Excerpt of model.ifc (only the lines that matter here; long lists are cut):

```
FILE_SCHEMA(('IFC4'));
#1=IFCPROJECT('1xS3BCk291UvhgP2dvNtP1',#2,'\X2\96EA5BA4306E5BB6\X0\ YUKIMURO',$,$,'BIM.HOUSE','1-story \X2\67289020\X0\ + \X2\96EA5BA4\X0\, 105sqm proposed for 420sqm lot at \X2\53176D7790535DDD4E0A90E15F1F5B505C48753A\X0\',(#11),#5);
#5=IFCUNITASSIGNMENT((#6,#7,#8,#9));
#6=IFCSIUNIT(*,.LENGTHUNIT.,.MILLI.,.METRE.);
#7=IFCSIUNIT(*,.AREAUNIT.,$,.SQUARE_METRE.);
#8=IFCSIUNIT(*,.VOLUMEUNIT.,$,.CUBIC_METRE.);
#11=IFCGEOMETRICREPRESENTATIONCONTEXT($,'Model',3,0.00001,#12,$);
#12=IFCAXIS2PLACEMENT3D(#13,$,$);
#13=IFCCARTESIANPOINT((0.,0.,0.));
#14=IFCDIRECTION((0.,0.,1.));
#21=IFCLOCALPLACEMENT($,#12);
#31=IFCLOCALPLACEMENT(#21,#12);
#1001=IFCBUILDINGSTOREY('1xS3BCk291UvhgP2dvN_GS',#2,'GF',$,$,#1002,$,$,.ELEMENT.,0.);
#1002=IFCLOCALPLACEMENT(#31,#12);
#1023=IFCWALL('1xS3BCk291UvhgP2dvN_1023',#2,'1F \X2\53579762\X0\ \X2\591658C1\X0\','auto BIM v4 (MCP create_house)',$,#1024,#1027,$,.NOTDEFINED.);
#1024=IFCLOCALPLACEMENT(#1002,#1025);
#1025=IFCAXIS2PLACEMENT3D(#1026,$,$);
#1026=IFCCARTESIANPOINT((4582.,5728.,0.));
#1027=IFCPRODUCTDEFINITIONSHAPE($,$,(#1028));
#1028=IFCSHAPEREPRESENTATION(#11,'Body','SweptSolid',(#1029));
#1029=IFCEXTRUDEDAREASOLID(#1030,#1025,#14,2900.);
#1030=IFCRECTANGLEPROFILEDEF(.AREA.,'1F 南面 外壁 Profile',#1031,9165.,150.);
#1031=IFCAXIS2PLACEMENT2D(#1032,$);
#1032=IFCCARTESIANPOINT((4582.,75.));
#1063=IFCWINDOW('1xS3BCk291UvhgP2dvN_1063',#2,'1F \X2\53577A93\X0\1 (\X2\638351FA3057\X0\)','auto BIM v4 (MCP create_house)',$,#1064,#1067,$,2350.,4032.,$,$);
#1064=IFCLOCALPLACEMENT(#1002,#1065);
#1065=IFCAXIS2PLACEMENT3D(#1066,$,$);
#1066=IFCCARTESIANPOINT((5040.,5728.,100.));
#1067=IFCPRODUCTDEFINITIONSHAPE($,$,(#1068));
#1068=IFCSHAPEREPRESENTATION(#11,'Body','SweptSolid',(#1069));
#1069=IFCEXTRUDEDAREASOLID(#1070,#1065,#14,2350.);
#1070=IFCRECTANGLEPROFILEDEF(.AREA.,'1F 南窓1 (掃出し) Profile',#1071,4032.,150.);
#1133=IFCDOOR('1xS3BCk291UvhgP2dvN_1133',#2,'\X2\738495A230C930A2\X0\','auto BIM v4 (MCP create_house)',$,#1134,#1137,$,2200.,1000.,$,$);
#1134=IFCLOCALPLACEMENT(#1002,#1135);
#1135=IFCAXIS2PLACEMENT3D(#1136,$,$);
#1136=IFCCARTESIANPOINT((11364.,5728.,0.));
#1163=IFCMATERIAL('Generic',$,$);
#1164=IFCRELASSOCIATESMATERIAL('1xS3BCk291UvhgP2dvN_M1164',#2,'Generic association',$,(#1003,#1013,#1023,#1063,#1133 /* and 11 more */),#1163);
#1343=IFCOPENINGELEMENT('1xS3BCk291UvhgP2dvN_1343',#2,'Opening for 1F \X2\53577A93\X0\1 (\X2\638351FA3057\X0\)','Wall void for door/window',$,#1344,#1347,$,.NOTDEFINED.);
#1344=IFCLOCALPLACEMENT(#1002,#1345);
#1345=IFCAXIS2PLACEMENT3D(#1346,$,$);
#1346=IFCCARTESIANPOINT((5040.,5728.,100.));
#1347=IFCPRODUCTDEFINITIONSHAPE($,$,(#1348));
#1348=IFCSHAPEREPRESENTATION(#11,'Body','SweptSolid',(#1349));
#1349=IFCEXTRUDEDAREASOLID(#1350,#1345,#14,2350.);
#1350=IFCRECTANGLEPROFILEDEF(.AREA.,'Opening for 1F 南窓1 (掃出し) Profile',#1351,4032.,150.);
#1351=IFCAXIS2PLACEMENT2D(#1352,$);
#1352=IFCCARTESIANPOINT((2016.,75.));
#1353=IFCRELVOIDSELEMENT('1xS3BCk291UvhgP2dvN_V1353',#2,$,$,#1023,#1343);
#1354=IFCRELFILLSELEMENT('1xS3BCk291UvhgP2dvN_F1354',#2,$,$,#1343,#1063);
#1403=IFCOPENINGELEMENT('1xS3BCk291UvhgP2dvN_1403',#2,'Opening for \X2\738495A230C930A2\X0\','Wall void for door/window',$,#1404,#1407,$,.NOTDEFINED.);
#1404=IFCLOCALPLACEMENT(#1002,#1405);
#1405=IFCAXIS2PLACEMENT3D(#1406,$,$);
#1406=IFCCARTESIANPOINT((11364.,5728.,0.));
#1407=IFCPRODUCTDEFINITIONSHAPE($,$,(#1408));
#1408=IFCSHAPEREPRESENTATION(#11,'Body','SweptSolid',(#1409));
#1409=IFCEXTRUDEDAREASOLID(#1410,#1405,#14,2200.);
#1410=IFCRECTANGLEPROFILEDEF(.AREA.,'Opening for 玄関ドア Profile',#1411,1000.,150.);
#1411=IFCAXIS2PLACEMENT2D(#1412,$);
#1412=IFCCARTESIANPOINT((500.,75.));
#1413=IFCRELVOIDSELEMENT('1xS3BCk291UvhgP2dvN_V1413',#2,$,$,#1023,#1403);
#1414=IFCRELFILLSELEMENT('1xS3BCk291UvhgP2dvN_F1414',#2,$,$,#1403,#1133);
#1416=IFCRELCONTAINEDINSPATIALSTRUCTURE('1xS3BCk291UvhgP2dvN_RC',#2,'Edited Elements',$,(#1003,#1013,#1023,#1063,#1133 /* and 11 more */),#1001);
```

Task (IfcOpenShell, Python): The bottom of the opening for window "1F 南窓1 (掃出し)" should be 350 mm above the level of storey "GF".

```python
import numpy as np
import ifcopenshell
import ifcopenshell.api.geometry
import ifcopenshell.geom
import ifcopenshell.util.element
import ifcopenshell.util.placement
import ifcopenshell.util.shape
import ifcopenshell.util.unit

model = ifcopenshell.open("model.ifc")
unit_scale = ifcopenshell.util.unit.calculate_unit_scale(model)

window = model.by_guid("1xS3BCk291UvhgP2dvN_1063")
opening = window.FillsVoids[0].RelatingOpeningElement
storey = ifcopenshell.util.element.get_container(window, ifc_class="IfcBuildingStorey")
level = ifcopenshell.util.placement.get_local_placement(storey.ObjectPlacement)[2, 3]

# The opening's origin need not be at the sill, so measure its lowest point.
shape = ifcopenshell.geom.create_shape(ifcopenshell.geom.settings(), opening)
bottom = ifcopenshell.util.shape.get_shape_bottom_elevation(shape, shape.geometry) / unit_scale
dz = level + 0.35 / unit_scale - bottom

shift = np.array([0.0, 0.0, dz])
# The window is not placed relative to its opening, so move both.
for product in (opening, window):
    matrix = ifcopenshell.util.placement.get_local_placement(product.ObjectPlacement)
    matrix[:3, 3] += shift
    ifcopenshell.api.geometry.edit_object_placement(model, product=product, matrix=matrix, is_si=False)

print(f"moved by {dz * unit_scale:+.3f} m")

model.write("model_v2.ifc")
```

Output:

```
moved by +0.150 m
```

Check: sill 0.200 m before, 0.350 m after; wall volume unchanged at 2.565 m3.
